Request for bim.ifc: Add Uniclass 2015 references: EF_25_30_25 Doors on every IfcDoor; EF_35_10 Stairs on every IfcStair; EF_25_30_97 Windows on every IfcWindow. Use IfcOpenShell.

First a look at what the model holds.

```python
import ifcopenshell

model = ifcopenshell.open("bim.ifc")
print(model.schema)
print("classifications:", [c.Name for c in model.by_type("IfcClassification")])
for ifc_class in ("IfcDoor", "IfcRoof", "IfcStair", "IfcWall", "IfcWindow"):
    print(ifc_class, len(model.by_type(ifc_class)))
```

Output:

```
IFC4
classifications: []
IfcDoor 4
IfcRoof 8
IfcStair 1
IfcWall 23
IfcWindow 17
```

```python
import ifcopenshell
import ifcopenshell.api.classification

model = ifcopenshell.open("bim.ifc")

system = ifcopenshell.api.classification.add_classification(model, classification="Uniclass 2015")

codes = {
    "IfcDoor": ("EF_25_30_25", "Doors"),
    "IfcStair": ("EF_35_10", "Stairs"),
    "IfcWindow": ("EF_25_30_97", "Windows"),
}
for ifc_class, (code, name) in codes.items():
    products = model.by_type(ifc_class)
    ifcopenshell.api.classification.add_reference(
        model, products=products, classification=system, identification=code, name=name
    )
    print(code, len(products))

model.write("bim_rev.ifc")
```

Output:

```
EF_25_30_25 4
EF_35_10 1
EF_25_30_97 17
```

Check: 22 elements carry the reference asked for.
